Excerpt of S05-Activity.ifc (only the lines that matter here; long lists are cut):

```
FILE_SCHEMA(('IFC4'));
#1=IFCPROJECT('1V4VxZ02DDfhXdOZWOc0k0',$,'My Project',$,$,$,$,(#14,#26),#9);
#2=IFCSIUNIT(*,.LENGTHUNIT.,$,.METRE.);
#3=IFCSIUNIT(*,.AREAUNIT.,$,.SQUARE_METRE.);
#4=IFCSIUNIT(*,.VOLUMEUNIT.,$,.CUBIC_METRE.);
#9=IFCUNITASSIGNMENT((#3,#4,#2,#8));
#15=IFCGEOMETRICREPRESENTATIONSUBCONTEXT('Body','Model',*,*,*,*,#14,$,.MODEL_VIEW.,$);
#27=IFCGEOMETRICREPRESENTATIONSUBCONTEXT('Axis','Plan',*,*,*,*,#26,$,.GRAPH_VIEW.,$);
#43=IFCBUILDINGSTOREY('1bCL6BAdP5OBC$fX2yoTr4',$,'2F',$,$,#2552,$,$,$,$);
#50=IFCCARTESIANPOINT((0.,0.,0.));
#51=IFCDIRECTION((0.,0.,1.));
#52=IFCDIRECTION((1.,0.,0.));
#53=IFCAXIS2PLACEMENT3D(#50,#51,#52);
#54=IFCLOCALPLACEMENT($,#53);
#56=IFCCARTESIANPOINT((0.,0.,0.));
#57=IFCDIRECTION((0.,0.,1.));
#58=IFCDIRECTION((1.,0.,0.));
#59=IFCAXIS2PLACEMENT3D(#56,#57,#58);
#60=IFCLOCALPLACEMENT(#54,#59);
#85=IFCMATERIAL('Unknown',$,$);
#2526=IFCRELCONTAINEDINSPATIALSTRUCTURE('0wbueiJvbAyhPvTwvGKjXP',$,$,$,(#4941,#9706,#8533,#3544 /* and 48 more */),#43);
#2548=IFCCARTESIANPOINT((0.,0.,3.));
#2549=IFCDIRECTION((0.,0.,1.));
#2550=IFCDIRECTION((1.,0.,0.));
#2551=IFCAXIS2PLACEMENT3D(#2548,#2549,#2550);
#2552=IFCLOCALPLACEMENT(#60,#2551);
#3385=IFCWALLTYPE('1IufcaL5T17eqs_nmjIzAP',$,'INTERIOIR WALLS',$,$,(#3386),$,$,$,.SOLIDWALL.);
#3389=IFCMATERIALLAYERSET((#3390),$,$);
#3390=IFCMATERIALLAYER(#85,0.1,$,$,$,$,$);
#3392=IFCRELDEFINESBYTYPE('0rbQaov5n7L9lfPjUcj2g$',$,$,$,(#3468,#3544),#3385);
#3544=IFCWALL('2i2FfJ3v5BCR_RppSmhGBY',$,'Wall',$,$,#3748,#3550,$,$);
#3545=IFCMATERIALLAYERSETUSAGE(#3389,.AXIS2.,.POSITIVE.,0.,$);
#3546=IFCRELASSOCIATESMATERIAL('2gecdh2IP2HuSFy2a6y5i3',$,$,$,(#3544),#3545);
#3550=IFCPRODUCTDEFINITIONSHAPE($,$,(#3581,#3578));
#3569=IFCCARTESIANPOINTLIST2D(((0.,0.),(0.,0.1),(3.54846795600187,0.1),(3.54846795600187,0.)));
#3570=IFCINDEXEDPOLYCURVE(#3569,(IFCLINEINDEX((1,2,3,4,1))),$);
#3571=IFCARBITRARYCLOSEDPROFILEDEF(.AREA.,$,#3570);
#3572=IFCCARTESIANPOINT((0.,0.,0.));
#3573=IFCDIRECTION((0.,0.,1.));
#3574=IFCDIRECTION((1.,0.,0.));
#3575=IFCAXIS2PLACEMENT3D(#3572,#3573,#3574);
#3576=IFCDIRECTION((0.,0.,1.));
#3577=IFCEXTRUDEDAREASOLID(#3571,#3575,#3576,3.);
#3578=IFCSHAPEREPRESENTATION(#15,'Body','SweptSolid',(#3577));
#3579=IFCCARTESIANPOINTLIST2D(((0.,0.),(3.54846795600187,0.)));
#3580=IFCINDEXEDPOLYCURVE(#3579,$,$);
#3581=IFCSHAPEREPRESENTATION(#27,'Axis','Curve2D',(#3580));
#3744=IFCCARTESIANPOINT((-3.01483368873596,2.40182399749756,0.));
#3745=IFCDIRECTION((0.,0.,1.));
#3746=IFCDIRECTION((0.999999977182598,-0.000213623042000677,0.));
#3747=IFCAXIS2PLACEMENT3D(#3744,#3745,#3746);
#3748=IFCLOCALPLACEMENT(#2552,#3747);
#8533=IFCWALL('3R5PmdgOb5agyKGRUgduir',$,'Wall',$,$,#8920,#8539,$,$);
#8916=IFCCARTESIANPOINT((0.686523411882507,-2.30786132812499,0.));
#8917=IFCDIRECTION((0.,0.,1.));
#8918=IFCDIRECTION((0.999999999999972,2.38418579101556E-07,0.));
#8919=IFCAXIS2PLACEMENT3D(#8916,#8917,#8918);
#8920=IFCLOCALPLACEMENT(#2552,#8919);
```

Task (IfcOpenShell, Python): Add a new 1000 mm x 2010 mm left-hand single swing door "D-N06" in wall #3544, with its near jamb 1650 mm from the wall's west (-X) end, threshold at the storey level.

```python
import numpy as np
import ifcopenshell
import ifcopenshell.api.feature
import ifcopenshell.api.geometry
import ifcopenshell.api.root
import ifcopenshell.api.spatial
import ifcopenshell.geom
import ifcopenshell.util.element
import ifcopenshell.util.placement
import ifcopenshell.util.representation
import ifcopenshell.util.shape
import ifcopenshell.util.unit

model = ifcopenshell.open("S05-Activity.ifc")
unit_scale = ifcopenshell.util.unit.calculate_unit_scale(model)
settings = ifcopenshell.geom.settings()


def volume(element):
    """Net volume in cubic metres, openings subtracted."""
    shape = ifcopenshell.geom.create_shape(settings, element)
    return ifcopenshell.util.shape.get_volume(shape.geometry)


wall = model.by_guid("2i2FfJ3v5BCR_RppSmhGBY")
storey = ifcopenshell.util.element.get_container(wall, ifc_class="IfcBuildingStorey")
context = ifcopenshell.util.representation.get_context(model, "Model", "Body", "MODEL_VIEW")
before = volume(wall)

width, height, from_end, sill = 1, 2.01, 1.65, 0.0  # metres

# The wall runs along its own X axis, and the end named is its -X end.
wall_shape = ifcopenshell.geom.create_shape(settings, wall)
x, y, z = ifcopenshell.util.shape.get_vertices(wall_shape.geometry).T
start = x.min() + from_end
face, thickness = float(y.min()), float(y.max() - y.min())
wall_matrix = ifcopenshell.util.placement.get_local_placement(wall.ObjectPlacement)
level = ifcopenshell.util.placement.get_local_placement(storey.ObjectPlacement)[2, 3]


def in_wall(x, y):
    """Placement at x, y metres in the wall's axes, at sill height."""
    matrix = wall_matrix.copy()
    matrix[:, 3] = wall_matrix @ np.array([x / unit_scale, y / unit_scale, 0.0, 1.0])
    matrix[2, 3] = level + sill / unit_scale
    return matrix


# Opening: a box that overshoots both wall faces by 50 mm.
opening = ifcopenshell.api.root.create_entity(model, ifc_class="IfcOpeningElement", predefined_type="OPENING")
box = ifcopenshell.api.geometry.add_wall_representation(
    model, context=context, length=width, height=height, thickness=thickness + 0.1
)
ifcopenshell.api.geometry.assign_representation(model, product=opening, representation=box)
ifcopenshell.api.geometry.edit_object_placement(model, product=opening, matrix=in_wall(start, face - 0.05), is_si=False)
ifcopenshell.api.feature.add_feature(model, feature=opening, element=wall)

door = ifcopenshell.api.root.create_entity(model, ifc_class="IfcDoor", name="D-N06", predefined_type="DOOR")
door.OverallWidth, door.OverallHeight = width / unit_scale, height / unit_scale
door.OperationType = "SINGLE_SWING_LEFT"
body = ifcopenshell.api.geometry.add_door_representation(
    model,
    context=context,
    overall_width=door.OverallWidth,
    overall_height=door.OverallHeight,
    operation_type="SINGLE_SWING_LEFT",
    lining_properties={"LiningDepth": thickness / unit_scale, "ThresholdDepth": thickness / unit_scale},
)
ifcopenshell.api.geometry.assign_representation(model, product=door, representation=body)
ifcopenshell.api.spatial.assign_container(model, products=[door], relating_structure=storey)
ifcopenshell.api.feature.add_filling(model, opening=opening, element=door)

# The lining spans the wall, so the door starts at the wall face.
ifcopenshell.api.geometry.edit_object_placement(model, product=door, matrix=in_wall(start, face), is_si=False)

after = volume(wall)

print(f"wall volume {before:.3f} -> {after:.3f} m3")

model.write("S05-Activity_edited.ifc")
```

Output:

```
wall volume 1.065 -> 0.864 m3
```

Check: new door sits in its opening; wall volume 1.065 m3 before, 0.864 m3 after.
